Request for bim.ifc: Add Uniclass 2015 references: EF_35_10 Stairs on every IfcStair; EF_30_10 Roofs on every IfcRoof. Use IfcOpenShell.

First a look at what the model holds.

```python
import ifcopenshell

model = ifcopenshell.open("bim.ifc")
print(model.schema)
print("classifications:", [c.Name for c in model.by_type("IfcClassification")])
for ifc_class in ("IfcDoor", "IfcRoof", "IfcStair", "IfcWall", "IfcWindow"):
    print(ifc_class, len(model.by_type(ifc_class)))
```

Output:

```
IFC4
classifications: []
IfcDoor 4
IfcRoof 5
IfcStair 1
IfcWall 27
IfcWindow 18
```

```python
import ifcopenshell
import ifcopenshell.api.classification

model = ifcopenshell.open("bim.ifc")

system = ifcopenshell.api.classification.add_classification(model, classification="Uniclass 2015")

codes = {
    "IfcStair": ("EF_35_10", "Stairs"),
    "IfcRoof": ("EF_30_10", "Roofs"),
}
for ifc_class, (code, name) in codes.items():
    products = model.by_type(ifc_class)
    ifcopenshell.api.classification.add_reference(
        model, products=products, classification=system, identification=code, name=name
    )
    print(code, len(products))

model.write("bim_edited.ifc")
```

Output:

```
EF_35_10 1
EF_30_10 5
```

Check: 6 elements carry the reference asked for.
